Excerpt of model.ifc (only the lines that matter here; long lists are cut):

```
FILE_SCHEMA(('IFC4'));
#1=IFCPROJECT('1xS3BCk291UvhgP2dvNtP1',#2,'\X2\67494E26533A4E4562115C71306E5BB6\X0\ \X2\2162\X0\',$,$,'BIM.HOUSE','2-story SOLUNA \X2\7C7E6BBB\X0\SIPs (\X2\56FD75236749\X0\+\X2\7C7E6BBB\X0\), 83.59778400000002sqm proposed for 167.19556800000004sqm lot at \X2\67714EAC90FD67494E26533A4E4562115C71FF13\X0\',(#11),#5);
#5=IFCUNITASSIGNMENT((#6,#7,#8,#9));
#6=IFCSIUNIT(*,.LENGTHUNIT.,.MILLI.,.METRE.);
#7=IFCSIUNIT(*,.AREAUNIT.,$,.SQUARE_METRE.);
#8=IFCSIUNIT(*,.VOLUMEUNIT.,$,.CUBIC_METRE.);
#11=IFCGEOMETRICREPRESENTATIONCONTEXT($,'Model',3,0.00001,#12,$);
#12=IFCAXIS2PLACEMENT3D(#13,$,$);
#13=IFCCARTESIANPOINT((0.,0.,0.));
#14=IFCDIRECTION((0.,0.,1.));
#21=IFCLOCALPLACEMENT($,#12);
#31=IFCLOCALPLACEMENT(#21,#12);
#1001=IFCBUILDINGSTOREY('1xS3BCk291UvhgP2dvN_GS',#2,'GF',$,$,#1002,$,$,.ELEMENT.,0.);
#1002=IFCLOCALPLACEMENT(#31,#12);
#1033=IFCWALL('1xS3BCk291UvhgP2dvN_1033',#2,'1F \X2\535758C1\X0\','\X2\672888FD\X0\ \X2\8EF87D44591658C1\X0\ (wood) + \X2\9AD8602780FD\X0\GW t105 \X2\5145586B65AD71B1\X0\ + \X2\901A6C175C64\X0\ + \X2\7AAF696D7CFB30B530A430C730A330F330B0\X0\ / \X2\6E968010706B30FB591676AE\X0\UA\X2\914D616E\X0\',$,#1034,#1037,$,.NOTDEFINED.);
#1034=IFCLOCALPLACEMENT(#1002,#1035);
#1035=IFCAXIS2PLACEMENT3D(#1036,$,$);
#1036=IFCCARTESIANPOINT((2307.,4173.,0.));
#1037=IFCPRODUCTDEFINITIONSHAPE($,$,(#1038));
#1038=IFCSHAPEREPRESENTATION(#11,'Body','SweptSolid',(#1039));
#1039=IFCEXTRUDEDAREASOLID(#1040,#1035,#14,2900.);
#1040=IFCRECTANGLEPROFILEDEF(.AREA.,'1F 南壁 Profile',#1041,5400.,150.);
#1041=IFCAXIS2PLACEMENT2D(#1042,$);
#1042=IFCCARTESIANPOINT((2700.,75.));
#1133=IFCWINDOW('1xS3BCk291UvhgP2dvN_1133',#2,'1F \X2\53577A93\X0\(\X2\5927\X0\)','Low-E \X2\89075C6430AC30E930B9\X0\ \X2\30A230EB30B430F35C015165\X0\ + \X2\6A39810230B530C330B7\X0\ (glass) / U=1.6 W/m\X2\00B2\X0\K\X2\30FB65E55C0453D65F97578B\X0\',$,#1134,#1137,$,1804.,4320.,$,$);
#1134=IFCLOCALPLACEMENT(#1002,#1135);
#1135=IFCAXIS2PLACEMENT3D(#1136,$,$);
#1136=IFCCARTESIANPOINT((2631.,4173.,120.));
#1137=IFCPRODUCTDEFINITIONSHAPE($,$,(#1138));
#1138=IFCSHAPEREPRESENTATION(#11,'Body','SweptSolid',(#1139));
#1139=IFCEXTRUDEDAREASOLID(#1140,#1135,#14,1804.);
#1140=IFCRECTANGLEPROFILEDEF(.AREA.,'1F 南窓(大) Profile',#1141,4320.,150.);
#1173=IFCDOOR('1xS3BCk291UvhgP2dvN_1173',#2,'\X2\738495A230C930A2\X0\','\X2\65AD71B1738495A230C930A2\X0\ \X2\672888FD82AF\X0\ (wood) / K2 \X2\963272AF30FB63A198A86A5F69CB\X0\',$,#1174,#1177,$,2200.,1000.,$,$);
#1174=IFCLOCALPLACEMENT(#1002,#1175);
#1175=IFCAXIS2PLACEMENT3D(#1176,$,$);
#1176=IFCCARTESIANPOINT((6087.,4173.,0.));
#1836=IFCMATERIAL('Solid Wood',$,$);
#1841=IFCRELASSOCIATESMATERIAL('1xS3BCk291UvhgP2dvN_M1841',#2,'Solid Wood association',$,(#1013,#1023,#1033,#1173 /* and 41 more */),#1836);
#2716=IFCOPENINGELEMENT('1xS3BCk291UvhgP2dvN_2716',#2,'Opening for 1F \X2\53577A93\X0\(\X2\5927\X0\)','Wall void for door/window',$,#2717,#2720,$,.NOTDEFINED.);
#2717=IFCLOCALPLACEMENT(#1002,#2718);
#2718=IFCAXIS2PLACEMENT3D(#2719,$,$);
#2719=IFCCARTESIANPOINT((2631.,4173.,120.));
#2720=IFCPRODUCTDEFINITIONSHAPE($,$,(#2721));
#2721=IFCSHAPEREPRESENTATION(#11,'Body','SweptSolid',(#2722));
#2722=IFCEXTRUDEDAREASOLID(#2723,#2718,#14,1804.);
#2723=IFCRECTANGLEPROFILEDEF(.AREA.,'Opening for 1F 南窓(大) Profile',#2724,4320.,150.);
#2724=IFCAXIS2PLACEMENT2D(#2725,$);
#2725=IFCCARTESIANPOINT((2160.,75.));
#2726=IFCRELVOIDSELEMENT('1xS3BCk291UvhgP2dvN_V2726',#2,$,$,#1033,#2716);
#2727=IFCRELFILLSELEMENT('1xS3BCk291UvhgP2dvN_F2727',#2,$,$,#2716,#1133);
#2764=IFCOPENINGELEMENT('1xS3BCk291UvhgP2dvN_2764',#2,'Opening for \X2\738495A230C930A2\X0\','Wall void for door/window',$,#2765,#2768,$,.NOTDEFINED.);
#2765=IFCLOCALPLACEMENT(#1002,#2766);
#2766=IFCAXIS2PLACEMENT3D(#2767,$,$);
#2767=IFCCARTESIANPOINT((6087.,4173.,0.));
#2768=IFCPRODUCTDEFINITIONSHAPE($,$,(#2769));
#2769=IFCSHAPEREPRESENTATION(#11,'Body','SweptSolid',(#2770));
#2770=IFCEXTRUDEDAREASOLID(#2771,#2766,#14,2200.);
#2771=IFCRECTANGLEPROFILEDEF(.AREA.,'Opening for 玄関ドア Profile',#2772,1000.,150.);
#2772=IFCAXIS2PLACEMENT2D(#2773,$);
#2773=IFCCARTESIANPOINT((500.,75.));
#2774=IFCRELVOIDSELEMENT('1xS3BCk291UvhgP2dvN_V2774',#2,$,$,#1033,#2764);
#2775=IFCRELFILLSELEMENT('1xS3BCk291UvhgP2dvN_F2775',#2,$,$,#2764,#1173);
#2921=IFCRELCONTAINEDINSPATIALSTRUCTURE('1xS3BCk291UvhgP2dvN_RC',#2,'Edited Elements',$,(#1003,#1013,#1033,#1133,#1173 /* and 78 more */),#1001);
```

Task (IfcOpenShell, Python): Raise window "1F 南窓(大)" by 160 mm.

```python
import numpy as np
import ifcopenshell
import ifcopenshell.api.geometry
import ifcopenshell.util.placement
import ifcopenshell.util.unit

model = ifcopenshell.open("model.ifc")
unit_scale = ifcopenshell.util.unit.calculate_unit_scale(model)

window = model.by_guid("1xS3BCk291UvhgP2dvN_1133")
opening = window.FillsVoids[0].RelatingOpeningElement
dz = 160.0

shift = np.array([0.0, 0.0, dz])
# The window is not placed relative to its opening, so move both.
for product in (opening, window):
    matrix = ifcopenshell.util.placement.get_local_placement(product.ObjectPlacement)
    matrix[:3, 3] += shift
    ifcopenshell.api.geometry.edit_object_placement(model, product=product, matrix=matrix, is_si=False)

print(f"moved by {dz * unit_scale:+.3f} m")

model.write("model_rev.ifc")
```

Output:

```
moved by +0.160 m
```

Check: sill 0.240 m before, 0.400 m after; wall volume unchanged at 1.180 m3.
